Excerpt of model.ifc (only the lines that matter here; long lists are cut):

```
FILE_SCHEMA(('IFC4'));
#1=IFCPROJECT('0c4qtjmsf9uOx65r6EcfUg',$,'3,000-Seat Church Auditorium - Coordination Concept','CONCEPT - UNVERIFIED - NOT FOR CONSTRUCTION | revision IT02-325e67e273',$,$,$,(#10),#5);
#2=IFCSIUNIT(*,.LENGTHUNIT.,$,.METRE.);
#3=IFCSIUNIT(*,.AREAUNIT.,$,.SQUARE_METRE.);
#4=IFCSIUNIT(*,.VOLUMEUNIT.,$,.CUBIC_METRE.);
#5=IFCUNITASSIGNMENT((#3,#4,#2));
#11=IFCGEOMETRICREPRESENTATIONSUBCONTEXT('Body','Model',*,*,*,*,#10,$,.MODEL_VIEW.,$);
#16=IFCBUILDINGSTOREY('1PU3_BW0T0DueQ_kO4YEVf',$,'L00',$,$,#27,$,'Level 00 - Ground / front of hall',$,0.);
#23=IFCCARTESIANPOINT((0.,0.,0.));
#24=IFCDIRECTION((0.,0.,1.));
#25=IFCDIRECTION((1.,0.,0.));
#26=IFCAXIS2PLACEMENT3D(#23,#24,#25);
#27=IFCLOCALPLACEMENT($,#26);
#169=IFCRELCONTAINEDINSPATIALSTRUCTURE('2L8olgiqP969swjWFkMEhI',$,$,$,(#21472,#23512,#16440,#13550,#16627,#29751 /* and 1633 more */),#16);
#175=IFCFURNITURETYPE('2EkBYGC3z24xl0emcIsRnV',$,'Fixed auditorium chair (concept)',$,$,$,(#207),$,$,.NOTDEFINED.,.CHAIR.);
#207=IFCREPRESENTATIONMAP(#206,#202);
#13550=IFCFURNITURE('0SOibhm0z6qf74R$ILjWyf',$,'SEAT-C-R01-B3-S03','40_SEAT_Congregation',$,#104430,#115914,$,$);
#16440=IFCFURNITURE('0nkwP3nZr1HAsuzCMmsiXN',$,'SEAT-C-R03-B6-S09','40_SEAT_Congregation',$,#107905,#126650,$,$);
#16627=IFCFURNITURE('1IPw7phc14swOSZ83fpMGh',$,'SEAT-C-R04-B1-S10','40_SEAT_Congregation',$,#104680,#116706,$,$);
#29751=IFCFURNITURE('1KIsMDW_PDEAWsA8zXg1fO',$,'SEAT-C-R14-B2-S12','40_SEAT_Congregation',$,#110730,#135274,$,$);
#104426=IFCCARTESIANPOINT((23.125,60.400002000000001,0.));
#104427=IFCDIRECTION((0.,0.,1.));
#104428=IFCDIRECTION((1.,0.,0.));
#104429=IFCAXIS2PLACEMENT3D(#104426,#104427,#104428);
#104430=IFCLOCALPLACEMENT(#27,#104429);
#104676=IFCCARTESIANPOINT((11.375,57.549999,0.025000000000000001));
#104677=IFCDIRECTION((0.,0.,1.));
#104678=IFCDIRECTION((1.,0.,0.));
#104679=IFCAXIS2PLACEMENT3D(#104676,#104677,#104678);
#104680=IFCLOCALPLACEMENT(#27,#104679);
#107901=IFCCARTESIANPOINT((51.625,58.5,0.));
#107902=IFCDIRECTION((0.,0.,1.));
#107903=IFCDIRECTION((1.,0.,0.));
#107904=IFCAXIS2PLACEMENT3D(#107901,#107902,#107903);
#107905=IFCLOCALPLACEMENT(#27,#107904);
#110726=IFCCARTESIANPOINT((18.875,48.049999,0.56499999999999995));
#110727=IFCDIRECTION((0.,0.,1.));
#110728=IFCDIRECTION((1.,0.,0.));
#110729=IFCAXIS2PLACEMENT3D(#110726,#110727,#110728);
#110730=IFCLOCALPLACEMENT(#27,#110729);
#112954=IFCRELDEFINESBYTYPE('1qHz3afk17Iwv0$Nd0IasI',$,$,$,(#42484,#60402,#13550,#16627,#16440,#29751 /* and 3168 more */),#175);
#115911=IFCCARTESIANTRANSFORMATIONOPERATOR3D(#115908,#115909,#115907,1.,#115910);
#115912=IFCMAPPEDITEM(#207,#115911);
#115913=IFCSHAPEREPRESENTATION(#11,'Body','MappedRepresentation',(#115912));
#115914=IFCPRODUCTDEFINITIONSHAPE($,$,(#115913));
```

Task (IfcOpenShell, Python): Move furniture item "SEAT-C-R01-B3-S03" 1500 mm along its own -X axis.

```python
import ifcopenshell
import ifcopenshell.api.geometry
import ifcopenshell.util.placement
import ifcopenshell.util.unit

model = ifcopenshell.open("model.ifc")
unit_scale = ifcopenshell.util.unit.calculate_unit_scale(model)

item = model.by_guid("0SOibhm0z6qf74R$ILjWyf")
matrix = ifcopenshell.util.placement.get_local_placement(item.ObjectPlacement)
matrix[:3, 3] -= matrix[:3, 0] * 1.5 / unit_scale
ifcopenshell.api.geometry.edit_object_placement(model, product=item, matrix=matrix, is_si=False)

print(ifcopenshell.util.placement.get_local_placement(item.ObjectPlacement).round(3) + 0.0)

model.write("model_updated.ifc")
```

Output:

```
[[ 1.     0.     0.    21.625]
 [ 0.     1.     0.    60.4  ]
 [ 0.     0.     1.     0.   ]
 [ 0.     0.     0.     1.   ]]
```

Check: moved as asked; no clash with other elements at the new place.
